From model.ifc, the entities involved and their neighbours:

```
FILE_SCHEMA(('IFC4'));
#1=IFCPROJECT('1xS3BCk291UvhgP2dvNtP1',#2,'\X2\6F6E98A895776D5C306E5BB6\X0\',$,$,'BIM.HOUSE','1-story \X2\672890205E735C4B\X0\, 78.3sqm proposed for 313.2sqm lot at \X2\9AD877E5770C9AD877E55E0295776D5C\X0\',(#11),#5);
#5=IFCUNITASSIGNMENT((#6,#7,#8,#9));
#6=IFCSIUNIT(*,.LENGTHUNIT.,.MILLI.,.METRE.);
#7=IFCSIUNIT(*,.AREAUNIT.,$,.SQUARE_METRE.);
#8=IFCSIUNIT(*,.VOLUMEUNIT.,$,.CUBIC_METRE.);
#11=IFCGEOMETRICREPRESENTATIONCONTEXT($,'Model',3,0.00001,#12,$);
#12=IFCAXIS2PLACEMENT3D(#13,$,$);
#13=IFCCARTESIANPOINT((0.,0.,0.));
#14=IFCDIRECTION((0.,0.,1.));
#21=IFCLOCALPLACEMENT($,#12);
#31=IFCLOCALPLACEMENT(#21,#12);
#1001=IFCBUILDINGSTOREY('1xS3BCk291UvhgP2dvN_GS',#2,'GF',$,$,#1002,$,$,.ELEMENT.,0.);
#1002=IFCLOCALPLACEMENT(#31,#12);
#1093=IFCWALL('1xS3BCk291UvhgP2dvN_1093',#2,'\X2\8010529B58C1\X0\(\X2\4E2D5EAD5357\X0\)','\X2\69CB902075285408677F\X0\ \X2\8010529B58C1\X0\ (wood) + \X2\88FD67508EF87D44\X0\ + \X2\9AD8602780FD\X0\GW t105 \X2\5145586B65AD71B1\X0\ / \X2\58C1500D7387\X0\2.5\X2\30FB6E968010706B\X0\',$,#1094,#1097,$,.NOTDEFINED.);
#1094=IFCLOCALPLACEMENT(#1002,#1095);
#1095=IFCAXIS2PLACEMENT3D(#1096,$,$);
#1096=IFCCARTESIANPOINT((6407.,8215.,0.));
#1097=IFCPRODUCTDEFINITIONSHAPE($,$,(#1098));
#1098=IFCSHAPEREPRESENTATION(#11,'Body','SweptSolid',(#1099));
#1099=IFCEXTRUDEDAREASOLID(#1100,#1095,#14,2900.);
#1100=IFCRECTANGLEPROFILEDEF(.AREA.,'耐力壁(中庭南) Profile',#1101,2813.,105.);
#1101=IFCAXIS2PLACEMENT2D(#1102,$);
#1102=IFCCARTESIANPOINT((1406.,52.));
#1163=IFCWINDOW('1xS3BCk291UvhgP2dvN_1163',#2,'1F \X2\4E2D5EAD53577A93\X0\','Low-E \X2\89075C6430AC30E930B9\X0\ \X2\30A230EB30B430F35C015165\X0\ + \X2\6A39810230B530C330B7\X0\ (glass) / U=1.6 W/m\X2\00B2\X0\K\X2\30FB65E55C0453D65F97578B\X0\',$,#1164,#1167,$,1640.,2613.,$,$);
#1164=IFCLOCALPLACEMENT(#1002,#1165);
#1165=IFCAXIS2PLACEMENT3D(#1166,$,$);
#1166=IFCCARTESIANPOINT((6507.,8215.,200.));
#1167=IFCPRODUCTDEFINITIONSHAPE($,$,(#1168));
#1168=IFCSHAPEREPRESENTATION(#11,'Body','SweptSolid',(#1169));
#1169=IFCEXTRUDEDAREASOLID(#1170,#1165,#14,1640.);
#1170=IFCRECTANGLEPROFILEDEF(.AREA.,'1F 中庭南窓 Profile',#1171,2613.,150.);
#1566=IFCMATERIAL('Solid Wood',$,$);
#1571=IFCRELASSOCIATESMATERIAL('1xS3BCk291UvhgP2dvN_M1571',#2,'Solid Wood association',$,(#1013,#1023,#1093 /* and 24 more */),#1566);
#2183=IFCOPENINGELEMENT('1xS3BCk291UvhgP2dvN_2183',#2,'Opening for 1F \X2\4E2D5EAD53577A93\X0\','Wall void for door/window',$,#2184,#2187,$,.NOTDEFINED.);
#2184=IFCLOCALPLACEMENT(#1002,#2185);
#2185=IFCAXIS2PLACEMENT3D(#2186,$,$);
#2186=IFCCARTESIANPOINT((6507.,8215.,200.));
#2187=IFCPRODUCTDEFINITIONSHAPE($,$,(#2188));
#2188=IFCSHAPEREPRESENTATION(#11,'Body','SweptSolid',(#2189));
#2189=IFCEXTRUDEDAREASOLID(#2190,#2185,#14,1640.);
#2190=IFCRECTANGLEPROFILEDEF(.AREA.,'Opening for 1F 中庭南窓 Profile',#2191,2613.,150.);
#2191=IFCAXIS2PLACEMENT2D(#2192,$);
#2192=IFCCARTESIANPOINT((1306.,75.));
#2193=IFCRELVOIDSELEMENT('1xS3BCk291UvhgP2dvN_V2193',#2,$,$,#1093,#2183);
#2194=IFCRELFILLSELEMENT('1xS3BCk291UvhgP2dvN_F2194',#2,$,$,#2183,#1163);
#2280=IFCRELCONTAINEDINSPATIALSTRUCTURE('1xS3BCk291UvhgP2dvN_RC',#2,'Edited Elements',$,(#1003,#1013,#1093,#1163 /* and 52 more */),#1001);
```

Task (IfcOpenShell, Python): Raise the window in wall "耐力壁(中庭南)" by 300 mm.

```python
import numpy as np
import ifcopenshell
import ifcopenshell.api.geometry
import ifcopenshell.util.placement
import ifcopenshell.util.unit

model = ifcopenshell.open("model.ifc")
unit_scale = ifcopenshell.util.unit.calculate_unit_scale(model)

window = model.by_guid("1xS3BCk291UvhgP2dvN_1163")
opening = window.FillsVoids[0].RelatingOpeningElement
dz = 300.0

shift = np.array([0.0, 0.0, dz])
# The window is not placed relative to its opening, so move both.
for product in (opening, window):
    matrix = ifcopenshell.util.placement.get_local_placement(product.ObjectPlacement)
    matrix[:3, 3] += shift
    ifcopenshell.api.geometry.edit_object_placement(model, product=product, matrix=matrix, is_si=False)

print(f"moved by {dz * unit_scale:+.3f} m")

model.write("model_v2.ifc")
```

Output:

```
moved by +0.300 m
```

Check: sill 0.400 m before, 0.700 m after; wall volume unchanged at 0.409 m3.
